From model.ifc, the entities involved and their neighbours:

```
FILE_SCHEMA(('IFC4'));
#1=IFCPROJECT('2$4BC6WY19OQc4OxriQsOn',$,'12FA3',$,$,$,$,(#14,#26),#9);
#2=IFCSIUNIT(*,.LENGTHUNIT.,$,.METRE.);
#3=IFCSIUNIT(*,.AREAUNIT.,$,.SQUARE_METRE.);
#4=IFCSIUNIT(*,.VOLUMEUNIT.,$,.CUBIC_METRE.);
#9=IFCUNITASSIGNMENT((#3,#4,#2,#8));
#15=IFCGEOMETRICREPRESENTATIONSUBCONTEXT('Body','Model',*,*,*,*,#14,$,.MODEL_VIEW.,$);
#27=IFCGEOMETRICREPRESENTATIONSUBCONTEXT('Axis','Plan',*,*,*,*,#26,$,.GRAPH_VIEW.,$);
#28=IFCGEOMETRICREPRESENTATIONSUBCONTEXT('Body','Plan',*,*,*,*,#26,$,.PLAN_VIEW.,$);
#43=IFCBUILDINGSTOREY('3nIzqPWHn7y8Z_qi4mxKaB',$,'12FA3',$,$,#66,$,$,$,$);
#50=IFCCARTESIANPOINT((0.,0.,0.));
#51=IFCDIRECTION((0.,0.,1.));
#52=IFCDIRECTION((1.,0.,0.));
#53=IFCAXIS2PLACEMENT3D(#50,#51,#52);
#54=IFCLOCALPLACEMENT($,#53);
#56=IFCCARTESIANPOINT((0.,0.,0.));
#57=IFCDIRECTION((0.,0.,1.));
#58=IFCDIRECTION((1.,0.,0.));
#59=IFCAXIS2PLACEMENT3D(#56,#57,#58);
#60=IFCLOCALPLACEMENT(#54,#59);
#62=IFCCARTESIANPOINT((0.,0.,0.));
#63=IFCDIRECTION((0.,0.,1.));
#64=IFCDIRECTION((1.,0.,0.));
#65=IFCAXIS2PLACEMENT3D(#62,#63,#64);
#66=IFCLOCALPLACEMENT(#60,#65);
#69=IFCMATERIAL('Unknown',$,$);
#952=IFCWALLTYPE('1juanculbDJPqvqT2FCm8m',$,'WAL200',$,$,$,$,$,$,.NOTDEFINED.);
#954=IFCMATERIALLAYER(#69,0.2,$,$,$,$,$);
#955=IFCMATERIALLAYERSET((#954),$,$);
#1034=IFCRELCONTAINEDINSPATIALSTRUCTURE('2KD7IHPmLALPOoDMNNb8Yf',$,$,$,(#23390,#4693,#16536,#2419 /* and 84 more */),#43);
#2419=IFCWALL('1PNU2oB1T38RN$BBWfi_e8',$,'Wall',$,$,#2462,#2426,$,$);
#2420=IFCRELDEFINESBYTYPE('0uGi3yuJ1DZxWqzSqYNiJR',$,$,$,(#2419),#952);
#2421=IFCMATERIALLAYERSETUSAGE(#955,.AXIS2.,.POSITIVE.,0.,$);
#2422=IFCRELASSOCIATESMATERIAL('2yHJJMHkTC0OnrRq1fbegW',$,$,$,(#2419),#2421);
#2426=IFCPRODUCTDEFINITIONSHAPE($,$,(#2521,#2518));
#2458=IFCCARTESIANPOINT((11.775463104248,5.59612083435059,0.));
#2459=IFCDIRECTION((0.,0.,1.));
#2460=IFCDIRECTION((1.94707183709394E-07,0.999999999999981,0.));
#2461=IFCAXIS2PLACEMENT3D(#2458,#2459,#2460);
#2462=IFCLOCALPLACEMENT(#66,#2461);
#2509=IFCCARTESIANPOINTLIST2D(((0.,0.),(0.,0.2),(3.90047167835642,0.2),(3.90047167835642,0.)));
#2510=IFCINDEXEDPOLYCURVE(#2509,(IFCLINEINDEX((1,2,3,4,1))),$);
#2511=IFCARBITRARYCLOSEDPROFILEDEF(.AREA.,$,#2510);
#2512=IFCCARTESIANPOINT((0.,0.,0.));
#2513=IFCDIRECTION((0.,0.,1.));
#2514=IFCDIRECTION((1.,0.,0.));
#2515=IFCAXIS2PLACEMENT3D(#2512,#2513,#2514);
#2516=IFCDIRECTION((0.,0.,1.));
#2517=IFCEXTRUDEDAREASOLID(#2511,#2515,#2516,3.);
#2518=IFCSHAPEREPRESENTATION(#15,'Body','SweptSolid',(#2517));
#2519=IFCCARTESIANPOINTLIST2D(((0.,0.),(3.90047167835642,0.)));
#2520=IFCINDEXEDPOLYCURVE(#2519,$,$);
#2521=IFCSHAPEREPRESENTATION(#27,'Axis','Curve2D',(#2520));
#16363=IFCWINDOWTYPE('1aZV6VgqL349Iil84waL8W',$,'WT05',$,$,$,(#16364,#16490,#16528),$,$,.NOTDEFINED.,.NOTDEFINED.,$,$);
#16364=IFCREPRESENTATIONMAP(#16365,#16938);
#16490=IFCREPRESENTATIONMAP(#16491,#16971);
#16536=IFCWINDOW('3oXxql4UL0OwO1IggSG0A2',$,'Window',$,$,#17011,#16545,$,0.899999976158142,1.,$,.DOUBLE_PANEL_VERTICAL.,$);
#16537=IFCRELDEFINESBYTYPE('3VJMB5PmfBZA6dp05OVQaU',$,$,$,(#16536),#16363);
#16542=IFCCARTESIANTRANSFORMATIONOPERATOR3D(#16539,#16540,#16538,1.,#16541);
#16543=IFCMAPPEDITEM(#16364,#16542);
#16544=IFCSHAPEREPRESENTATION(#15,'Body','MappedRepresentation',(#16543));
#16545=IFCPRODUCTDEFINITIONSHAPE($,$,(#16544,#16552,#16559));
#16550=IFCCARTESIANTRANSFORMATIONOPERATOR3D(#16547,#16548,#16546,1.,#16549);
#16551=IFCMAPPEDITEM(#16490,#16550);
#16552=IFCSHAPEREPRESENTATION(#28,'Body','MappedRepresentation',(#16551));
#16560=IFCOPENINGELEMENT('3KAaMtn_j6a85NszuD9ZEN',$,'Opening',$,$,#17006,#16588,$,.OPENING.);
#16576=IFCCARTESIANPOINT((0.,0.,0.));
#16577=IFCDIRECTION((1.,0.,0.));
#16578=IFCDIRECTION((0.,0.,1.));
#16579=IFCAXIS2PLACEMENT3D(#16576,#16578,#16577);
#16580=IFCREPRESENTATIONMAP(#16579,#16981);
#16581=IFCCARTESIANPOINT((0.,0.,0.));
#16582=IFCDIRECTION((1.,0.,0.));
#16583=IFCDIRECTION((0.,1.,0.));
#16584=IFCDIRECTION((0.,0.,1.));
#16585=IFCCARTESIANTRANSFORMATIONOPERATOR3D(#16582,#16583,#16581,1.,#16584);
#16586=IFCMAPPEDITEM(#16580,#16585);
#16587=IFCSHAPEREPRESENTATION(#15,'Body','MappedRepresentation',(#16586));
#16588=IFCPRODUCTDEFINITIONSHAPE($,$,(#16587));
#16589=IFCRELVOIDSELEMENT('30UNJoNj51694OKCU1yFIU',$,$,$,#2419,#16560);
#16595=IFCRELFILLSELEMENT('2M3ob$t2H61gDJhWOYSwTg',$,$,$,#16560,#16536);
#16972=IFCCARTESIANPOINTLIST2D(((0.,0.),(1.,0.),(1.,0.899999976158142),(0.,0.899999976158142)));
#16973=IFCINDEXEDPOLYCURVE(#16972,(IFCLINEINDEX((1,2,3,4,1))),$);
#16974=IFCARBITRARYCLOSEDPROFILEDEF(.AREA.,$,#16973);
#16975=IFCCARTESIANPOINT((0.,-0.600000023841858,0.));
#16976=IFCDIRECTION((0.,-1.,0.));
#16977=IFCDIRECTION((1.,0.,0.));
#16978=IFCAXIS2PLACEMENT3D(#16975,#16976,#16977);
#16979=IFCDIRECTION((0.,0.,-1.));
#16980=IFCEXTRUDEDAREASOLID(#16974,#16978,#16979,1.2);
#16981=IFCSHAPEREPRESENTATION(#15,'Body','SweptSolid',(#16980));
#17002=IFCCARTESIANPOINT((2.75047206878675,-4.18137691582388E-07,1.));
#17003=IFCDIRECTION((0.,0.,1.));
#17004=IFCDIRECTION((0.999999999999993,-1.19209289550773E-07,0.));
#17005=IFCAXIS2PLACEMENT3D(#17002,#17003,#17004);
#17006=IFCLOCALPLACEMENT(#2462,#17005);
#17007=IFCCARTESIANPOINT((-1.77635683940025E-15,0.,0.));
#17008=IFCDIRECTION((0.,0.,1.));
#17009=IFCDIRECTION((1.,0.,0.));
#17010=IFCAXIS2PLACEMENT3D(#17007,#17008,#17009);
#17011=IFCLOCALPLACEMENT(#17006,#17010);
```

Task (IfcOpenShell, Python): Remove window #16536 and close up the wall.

```python
import ifcopenshell
import ifcopenshell.api.feature
import ifcopenshell.api.root
import ifcopenshell.geom
import ifcopenshell.util.shape

model = ifcopenshell.open("model.ifc")
settings = ifcopenshell.geom.settings()


def volume(element):
    """Net volume in cubic metres, openings subtracted."""
    shape = ifcopenshell.geom.create_shape(settings, element)
    return ifcopenshell.util.shape.get_volume(shape.geometry)


window = model.by_id(16536)
opening = window.FillsVoids[0].RelatingOpeningElement
wall = opening.VoidsElements[0].RelatingBuildingElement
before = volume(wall)

ifcopenshell.api.root.remove_product(model, product=window)
ifcopenshell.api.feature.remove_feature(model, feature=opening)

after = volume(wall)

print(f"wall volume {before:.3f} -> {after:.3f} m3")

model.write("model_rev.ifc")
```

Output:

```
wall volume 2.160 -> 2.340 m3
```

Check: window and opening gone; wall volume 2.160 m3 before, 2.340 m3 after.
